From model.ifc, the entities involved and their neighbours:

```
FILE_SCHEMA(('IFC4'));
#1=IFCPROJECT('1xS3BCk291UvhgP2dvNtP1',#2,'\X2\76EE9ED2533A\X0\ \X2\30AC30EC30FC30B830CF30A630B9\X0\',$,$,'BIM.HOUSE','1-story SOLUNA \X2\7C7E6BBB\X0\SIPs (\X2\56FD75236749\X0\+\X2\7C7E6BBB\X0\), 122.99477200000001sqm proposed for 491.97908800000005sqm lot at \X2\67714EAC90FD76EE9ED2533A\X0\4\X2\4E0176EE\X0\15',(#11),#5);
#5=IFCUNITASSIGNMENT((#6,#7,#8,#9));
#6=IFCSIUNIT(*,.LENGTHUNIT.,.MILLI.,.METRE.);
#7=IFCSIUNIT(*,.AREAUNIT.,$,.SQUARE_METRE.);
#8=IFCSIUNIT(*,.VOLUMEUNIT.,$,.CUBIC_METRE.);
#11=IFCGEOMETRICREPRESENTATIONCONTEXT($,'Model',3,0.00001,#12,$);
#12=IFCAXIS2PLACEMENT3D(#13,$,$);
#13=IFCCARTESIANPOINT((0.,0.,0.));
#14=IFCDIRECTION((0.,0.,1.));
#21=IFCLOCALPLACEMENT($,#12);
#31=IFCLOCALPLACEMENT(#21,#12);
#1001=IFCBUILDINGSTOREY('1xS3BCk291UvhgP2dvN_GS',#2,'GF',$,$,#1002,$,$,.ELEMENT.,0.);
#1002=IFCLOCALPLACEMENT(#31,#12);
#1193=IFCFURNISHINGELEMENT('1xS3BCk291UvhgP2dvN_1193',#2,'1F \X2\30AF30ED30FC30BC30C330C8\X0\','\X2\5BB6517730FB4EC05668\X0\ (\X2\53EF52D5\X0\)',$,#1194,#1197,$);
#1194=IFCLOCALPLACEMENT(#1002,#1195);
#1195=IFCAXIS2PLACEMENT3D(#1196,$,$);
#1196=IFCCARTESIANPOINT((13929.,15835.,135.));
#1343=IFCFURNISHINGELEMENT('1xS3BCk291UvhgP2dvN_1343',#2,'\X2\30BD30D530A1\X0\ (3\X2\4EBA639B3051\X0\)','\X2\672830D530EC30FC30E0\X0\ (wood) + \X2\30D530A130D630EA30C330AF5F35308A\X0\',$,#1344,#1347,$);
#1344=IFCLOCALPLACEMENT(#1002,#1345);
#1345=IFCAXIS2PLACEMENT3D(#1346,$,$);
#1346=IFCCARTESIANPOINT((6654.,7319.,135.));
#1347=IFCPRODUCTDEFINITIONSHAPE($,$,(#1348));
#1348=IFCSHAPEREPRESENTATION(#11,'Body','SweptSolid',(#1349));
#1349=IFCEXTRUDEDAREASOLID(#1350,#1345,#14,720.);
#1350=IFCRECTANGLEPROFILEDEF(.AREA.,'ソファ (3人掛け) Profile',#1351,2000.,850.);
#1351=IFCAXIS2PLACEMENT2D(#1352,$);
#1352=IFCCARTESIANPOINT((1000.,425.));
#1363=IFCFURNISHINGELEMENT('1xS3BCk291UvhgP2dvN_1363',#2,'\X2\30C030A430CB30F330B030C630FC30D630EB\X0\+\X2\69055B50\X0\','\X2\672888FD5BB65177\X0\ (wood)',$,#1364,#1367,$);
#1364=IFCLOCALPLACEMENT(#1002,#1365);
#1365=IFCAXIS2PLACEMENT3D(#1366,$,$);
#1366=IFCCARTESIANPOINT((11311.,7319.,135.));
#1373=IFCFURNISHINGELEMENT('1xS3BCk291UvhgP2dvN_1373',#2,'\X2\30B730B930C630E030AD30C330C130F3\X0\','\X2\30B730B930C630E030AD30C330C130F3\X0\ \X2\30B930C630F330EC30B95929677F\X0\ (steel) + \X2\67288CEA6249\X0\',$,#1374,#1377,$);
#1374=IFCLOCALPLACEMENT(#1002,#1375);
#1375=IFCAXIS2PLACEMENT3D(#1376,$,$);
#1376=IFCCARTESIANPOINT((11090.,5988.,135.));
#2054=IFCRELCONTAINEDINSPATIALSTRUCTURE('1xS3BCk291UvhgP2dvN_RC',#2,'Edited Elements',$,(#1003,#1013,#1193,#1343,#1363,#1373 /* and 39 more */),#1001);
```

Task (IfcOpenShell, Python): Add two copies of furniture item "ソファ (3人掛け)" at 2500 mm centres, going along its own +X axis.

```python
import ifcopenshell
import ifcopenshell.api.geometry
import ifcopenshell.api.root
import ifcopenshell.util.element
import ifcopenshell.util.placement

model = ifcopenshell.open("model.ifc")


def reuse_history(source, copy):
    """copy_class also copies each property set's owner history, people and application; keep the originals."""
    for rel in copy.IsDefinedBy:
        if rel.is_a("IfcRelDefinesByProperties") and (history := rel.RelatingPropertyDefinition.OwnerHistory):
            rel.RelatingPropertyDefinition.OwnerHistory = source.OwnerHistory
            ifcopenshell.util.element.remove_deep2(model, history)


source = model.by_guid("1xS3BCk291UvhgP2dvN_1343")
base = ifcopenshell.util.placement.get_local_placement(source.ObjectPlacement)
step = base[:3, 0] * 2500.0

for i in range(1, 3):
    copy = ifcopenshell.api.root.copy_class(model, product=source)
    copy.Representation = ifcopenshell.util.element.copy_deep(
        model, source.Representation, exclude=["IfcGeometricRepresentationContext", "IfcRepresentationMap"]
    )
    reuse_history(source, copy)
    matrix = base.copy()
    matrix[:3, 3] += i * step
    print("added at", matrix[:3, 3].round(3) + 0.0)
    ifcopenshell.api.geometry.edit_object_placement(model, product=copy, matrix=matrix, is_si=False)

model.write("model_v2.ifc")
```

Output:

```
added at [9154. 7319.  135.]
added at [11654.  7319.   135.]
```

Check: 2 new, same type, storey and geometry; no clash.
